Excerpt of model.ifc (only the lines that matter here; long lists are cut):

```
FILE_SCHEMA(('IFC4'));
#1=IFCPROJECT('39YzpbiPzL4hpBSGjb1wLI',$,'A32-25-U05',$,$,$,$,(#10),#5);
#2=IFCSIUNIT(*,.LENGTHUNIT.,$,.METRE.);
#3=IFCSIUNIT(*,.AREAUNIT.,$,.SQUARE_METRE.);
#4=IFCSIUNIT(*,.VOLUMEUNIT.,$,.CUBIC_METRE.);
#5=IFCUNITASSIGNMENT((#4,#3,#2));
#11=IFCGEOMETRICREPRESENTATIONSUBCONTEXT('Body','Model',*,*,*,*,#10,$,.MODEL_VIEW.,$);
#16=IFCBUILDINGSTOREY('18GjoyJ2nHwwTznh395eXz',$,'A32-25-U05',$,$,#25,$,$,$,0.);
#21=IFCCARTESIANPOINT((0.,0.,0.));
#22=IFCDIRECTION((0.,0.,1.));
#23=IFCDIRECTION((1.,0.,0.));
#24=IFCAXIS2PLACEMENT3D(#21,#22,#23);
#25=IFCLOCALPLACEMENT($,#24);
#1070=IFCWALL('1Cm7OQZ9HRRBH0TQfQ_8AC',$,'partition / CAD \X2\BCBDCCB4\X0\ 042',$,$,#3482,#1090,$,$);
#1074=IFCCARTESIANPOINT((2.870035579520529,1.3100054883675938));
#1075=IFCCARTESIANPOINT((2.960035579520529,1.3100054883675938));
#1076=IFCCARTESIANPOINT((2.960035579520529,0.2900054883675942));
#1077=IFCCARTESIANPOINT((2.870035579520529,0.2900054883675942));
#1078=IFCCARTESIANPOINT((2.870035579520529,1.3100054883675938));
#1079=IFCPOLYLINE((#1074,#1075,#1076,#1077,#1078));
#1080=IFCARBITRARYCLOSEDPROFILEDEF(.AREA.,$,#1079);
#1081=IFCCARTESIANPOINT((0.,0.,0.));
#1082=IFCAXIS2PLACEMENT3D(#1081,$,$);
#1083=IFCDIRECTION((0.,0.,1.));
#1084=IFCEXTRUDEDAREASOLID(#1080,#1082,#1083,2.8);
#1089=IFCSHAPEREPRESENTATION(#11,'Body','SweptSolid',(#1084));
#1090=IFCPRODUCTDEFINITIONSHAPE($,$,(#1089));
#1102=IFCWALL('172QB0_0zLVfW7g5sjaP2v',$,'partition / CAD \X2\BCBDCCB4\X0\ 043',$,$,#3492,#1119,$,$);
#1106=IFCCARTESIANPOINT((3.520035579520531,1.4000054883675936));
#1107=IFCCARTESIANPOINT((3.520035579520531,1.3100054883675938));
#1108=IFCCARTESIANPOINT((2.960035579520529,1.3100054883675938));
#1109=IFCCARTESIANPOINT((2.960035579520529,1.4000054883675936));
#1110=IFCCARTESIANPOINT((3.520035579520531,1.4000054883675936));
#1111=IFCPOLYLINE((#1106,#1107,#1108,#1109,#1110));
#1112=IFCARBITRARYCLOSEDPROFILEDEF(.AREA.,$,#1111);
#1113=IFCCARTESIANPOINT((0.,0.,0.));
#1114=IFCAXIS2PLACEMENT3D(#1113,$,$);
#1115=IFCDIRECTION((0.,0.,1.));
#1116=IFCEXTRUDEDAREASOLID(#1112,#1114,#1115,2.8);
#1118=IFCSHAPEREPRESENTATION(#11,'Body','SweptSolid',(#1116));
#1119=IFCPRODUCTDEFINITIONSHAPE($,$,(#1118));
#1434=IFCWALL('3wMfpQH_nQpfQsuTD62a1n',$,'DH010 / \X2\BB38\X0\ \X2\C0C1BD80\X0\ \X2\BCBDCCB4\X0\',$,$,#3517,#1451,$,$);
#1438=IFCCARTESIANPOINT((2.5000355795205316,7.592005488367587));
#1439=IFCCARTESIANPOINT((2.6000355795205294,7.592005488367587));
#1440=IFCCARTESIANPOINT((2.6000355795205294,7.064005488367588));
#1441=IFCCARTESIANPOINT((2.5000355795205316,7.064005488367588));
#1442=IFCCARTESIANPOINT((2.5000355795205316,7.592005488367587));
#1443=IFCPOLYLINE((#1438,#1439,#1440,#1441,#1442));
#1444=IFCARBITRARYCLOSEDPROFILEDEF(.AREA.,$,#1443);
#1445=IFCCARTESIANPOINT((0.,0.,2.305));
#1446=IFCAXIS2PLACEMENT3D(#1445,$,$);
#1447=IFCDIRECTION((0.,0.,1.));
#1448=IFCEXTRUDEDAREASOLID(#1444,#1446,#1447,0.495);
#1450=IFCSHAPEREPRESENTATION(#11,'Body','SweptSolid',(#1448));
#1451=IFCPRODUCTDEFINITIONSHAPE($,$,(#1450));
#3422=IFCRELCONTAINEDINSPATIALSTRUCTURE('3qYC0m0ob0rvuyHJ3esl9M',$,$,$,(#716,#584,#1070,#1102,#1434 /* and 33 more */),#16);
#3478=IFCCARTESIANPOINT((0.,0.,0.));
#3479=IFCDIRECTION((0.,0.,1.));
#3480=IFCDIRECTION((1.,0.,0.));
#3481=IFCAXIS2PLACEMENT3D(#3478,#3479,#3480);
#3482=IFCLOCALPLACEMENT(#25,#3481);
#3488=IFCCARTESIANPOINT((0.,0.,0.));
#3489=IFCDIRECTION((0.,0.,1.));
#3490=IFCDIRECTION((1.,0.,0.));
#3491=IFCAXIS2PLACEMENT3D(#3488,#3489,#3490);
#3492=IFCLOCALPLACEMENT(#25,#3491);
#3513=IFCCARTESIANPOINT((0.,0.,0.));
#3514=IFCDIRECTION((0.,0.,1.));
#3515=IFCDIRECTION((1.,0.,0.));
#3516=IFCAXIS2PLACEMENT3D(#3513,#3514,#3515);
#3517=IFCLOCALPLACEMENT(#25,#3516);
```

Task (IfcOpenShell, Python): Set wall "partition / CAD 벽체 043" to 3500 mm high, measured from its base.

```python
import ifcopenshell
import ifcopenshell.geom
import ifcopenshell.util.representation
import ifcopenshell.util.shape

model = ifcopenshell.open("model.ifc")
settings = ifcopenshell.geom.settings()


def volume(element):
    """Net volume in cubic metres, openings subtracted."""
    shape = ifcopenshell.geom.create_shape(settings, element)
    return ifcopenshell.util.shape.get_volume(shape.geometry)


wall = model.by_id(1102)
before = volume(wall)

body = ifcopenshell.util.representation.get_representation(wall, "Model", "Body")
solid = body.Items[0]
old_height = solid.Depth
solid.Depth = 3.5
after = volume(wall)

print(f"height {old_height:g} -> {solid.Depth:g}, volume {before:.3f} -> {after:.3f} m3")

model.write("model_updated.ifc")
```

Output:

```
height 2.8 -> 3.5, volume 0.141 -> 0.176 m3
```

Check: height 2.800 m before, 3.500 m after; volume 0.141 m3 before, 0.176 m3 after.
